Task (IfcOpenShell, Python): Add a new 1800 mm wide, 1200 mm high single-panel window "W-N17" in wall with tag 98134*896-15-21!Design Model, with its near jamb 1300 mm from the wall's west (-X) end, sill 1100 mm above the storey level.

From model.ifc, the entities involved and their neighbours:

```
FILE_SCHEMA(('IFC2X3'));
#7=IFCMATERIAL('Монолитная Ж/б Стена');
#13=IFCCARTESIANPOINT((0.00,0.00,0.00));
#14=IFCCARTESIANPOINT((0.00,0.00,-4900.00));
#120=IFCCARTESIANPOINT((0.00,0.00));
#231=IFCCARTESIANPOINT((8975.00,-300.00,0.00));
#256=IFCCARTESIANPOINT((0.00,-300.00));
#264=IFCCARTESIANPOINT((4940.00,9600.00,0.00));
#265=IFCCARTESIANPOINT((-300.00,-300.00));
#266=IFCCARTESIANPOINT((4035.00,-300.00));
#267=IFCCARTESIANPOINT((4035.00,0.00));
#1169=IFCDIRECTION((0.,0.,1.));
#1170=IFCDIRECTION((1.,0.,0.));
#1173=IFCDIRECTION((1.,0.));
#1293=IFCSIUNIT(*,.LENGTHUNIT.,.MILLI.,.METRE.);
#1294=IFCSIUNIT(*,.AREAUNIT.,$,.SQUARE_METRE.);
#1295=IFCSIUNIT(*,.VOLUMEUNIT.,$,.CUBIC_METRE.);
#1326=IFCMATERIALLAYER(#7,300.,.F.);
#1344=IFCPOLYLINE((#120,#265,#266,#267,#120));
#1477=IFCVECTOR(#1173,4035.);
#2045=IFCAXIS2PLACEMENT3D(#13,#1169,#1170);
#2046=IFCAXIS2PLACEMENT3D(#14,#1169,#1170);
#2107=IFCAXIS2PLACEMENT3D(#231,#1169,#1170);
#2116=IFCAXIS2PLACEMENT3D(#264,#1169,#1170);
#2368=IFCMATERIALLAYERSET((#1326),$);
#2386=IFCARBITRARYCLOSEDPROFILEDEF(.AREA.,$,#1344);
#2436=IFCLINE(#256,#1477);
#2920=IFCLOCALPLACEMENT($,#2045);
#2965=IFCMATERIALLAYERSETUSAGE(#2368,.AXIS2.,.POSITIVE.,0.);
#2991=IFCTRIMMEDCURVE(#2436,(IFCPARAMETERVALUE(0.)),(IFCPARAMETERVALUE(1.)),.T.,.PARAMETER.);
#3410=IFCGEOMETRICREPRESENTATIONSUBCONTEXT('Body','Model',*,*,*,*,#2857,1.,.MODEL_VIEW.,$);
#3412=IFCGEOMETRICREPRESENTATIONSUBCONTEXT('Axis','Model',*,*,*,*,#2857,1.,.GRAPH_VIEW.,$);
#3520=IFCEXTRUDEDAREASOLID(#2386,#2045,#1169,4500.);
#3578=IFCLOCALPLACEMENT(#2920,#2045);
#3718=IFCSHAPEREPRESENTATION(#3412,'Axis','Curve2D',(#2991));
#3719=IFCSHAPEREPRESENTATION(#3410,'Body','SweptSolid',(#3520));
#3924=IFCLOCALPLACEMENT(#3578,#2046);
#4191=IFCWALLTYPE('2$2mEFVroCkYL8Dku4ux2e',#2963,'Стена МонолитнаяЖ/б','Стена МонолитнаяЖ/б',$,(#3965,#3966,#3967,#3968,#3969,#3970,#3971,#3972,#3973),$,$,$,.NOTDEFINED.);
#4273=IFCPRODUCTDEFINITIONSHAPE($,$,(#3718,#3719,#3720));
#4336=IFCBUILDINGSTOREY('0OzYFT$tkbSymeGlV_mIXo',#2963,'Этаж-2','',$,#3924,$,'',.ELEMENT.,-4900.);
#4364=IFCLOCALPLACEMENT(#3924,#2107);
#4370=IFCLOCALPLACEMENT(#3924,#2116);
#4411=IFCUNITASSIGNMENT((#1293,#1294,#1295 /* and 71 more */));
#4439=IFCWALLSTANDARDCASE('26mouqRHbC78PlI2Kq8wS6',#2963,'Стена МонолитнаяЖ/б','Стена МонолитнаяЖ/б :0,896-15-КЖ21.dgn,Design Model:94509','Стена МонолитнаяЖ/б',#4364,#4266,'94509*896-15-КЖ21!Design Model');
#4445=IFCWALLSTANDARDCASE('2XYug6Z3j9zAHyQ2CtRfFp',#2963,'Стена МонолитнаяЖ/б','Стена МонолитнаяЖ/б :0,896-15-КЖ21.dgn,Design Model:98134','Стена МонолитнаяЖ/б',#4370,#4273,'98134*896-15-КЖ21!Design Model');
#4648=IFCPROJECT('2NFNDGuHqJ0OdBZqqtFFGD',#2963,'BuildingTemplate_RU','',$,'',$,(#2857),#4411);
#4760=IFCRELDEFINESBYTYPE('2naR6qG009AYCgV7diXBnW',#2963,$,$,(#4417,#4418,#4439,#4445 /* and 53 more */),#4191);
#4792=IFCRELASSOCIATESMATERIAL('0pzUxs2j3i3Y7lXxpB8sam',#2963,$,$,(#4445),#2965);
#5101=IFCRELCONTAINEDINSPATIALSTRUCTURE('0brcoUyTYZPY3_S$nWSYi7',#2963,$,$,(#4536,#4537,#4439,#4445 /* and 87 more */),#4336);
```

```python
import numpy as np
import ifcopenshell
import ifcopenshell.api.feature
import ifcopenshell.api.geometry
import ifcopenshell.api.root
import ifcopenshell.api.spatial
import ifcopenshell.api.type
import ifcopenshell.geom
import ifcopenshell.util.element
import ifcopenshell.util.placement
import ifcopenshell.util.representation
import ifcopenshell.util.shape
import ifcopenshell.util.unit

model = ifcopenshell.open("model.ifc")
unit_scale = ifcopenshell.util.unit.calculate_unit_scale(model)
settings = ifcopenshell.geom.settings()


def volume(element):
    """Net volume in cubic metres, openings subtracted."""
    shape = ifcopenshell.geom.create_shape(settings, element)
    return ifcopenshell.util.shape.get_volume(shape.geometry)


wall = model.by_id(4445)
storey = ifcopenshell.util.element.get_container(wall, ifc_class="IfcBuildingStorey")
context = ifcopenshell.util.representation.get_context(model, "Model", "Body", "MODEL_VIEW")
before = volume(wall)

width, height, from_end, sill = 1.8, 1.2, 1.3, 1.1  # metres

# The wall runs along its own X axis, and the end named is its -X end.
wall_shape = ifcopenshell.geom.create_shape(settings, wall)
x, y, z = ifcopenshell.util.shape.get_vertices(wall_shape.geometry).T
start = x.min() + from_end
face, thickness = float(y.min()), float(y.max() - y.min())
wall_matrix = ifcopenshell.util.placement.get_local_placement(wall.ObjectPlacement)
level = ifcopenshell.util.placement.get_local_placement(storey.ObjectPlacement)[2, 3]


def in_wall(x, y):
    """Placement at x, y metres in the wall's axes, at sill height."""
    matrix = wall_matrix.copy()
    matrix[:, 3] = wall_matrix @ np.array([x / unit_scale, y / unit_scale, 0.0, 1.0])
    matrix[2, 3] = level + sill / unit_scale
    return matrix


# Opening: a box that overshoots both wall faces by 50 mm.
opening = ifcopenshell.api.root.create_entity(model, ifc_class="IfcOpeningElement")
box = ifcopenshell.api.geometry.add_wall_representation(
    model, context=context, length=width, height=height, thickness=thickness + 0.1
)
ifcopenshell.api.geometry.assign_representation(model, product=opening, representation=box)
ifcopenshell.api.geometry.edit_object_placement(model, product=opening, matrix=in_wall(start, face - 0.05), is_si=False)
ifcopenshell.api.feature.add_feature(model, feature=opening, element=wall)

window = ifcopenshell.api.root.create_entity(model, ifc_class="IfcWindow", name="W-N17")
window.OverallWidth, window.OverallHeight = width / unit_scale, height / unit_scale
body = ifcopenshell.api.geometry.add_window_representation(
    model,
    context=context,
    overall_width=window.OverallWidth,
    overall_height=window.OverallHeight,
    partition_type="SINGLE_PANEL",
)
ifcopenshell.api.geometry.assign_representation(model, product=window, representation=body)
ifcopenshell.api.spatial.assign_container(model, products=[window], relating_structure=storey)
fills = ifcopenshell.api.feature.add_filling(model, opening=opening, element=window)
fills.OwnerHistory = window.OwnerHistory  # required in IFC2X3

# IFC2X3 keeps the operation on the window style.
style = ifcopenshell.api.root.create_entity(model, ifc_class="IfcWindowStyle", name="W-N17")
style.OperationType, style.ConstructionType = "SINGLE_PANEL", "NOTDEFINED"
style.ParameterTakesPrecedence = style.Sizeable = False
ifcopenshell.api.type.assign_type(model, related_objects=[window], relating_type=style)

# Centre the window in the wall's thickness.
ifcopenshell.api.geometry.edit_object_placement(model, product=window, matrix=in_wall(start, face), is_si=False)
window_shape = ifcopenshell.geom.create_shape(settings, window)
depth = ifcopenshell.util.shape.get_vertices(window_shape.geometry)[:, 1]
offset = face + thickness / 2 - (depth.min() + depth.max()) / 2
ifcopenshell.api.geometry.edit_object_placement(model, product=window, matrix=in_wall(start, offset), is_si=False)

after = volume(wall)

print(f"wall volume {before:.3f} -> {after:.3f} m3")

model.write("model_updated.ifc")
```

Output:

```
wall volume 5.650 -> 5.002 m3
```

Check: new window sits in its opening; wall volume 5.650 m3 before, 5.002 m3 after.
